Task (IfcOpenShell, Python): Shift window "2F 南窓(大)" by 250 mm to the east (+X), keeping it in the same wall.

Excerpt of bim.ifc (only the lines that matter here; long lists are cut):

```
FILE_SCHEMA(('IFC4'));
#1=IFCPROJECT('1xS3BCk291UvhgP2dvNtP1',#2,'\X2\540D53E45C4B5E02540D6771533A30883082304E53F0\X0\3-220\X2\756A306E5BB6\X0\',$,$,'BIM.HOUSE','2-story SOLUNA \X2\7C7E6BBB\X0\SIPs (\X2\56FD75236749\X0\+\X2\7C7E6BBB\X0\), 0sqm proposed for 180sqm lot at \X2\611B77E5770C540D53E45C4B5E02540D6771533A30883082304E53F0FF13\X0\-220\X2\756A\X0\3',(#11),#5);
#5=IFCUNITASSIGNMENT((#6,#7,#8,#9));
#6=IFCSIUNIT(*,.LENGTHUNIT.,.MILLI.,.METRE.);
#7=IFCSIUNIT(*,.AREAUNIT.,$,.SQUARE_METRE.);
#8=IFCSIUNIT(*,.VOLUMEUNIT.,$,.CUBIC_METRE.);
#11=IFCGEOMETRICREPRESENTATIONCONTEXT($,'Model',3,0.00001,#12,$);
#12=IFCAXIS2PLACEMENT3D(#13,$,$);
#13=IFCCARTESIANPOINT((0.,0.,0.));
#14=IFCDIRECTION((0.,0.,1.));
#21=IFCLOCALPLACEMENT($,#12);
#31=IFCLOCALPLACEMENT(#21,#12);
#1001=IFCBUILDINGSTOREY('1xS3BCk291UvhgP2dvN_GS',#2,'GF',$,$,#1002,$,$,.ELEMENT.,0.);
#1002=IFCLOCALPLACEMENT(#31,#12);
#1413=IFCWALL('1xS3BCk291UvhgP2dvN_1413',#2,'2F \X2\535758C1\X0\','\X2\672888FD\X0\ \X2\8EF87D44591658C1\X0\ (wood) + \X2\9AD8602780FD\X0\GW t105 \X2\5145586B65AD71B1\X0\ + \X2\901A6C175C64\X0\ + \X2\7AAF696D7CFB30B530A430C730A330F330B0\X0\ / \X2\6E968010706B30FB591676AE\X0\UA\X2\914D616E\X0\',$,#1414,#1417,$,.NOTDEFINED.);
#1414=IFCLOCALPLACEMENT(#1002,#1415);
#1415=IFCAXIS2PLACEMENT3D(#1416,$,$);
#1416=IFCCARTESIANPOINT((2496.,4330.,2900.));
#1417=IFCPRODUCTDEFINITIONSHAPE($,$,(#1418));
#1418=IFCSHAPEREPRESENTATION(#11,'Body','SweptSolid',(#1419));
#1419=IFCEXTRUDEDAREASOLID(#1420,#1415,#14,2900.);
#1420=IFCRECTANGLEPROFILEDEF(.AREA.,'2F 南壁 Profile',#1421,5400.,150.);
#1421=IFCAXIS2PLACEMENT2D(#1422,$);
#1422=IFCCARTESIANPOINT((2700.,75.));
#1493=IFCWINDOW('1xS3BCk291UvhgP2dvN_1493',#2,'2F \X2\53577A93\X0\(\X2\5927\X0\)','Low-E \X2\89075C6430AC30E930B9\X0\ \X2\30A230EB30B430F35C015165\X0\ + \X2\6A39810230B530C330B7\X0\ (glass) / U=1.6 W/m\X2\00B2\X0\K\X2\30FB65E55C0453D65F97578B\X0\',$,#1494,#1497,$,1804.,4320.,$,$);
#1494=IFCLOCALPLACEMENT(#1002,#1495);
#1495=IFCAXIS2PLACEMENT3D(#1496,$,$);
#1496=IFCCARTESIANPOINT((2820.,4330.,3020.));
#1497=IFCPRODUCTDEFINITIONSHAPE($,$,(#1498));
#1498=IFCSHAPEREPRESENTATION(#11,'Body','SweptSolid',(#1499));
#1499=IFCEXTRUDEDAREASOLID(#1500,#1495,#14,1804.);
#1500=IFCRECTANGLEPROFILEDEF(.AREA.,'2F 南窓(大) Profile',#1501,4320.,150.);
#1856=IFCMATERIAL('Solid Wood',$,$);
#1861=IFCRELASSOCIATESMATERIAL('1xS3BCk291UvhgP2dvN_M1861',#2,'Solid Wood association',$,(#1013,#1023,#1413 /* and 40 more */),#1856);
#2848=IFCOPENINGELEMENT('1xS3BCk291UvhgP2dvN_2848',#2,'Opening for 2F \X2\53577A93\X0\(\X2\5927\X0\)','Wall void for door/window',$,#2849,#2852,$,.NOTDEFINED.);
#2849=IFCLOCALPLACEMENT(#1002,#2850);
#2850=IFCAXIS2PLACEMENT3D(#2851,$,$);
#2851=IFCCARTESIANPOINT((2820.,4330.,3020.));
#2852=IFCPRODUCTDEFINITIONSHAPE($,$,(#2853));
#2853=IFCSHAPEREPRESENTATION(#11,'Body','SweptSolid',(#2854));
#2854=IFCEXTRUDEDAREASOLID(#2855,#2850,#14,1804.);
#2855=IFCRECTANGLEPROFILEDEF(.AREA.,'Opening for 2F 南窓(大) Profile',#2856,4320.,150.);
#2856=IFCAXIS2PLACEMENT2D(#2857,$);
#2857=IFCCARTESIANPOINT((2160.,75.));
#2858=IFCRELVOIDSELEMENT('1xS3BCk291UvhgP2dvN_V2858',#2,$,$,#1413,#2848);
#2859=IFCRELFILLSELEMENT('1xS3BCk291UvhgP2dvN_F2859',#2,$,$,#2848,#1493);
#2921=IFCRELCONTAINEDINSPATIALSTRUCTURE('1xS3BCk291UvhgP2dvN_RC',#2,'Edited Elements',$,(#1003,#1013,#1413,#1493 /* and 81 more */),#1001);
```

```python
import ifcopenshell
import ifcopenshell.api.geometry
import ifcopenshell.util.placement
import ifcopenshell.util.unit

model = ifcopenshell.open("bim.ifc")
unit_scale = ifcopenshell.util.unit.calculate_unit_scale(model)

window = model.by_guid("1xS3BCk291UvhgP2dvN_1493")
opening = window.FillsVoids[0].RelatingOpeningElement
wall = opening.VoidsElements[0].RelatingBuildingElement

wall_matrix = ifcopenshell.util.placement.get_local_placement(wall.ObjectPlacement)
shift = wall_matrix[:3, 0] * 0.25 / unit_scale
before = ifcopenshell.util.placement.get_local_placement(window.ObjectPlacement)[:3, 3].copy()

# The window is not placed relative to its opening, so move both.
for product in (opening, window):
    matrix = ifcopenshell.util.placement.get_local_placement(product.ObjectPlacement)
    matrix[:3, 3] += shift
    ifcopenshell.api.geometry.edit_object_placement(model, product=product, matrix=matrix, is_si=False)

after = ifcopenshell.util.placement.get_local_placement(window.ObjectPlacement)[:3, 3]
print("window moved by", (after - before).round(3) + 0.0)

model.write("bim_updated.ifc")
```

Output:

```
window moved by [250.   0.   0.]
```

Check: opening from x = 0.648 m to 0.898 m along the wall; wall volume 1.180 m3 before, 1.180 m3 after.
